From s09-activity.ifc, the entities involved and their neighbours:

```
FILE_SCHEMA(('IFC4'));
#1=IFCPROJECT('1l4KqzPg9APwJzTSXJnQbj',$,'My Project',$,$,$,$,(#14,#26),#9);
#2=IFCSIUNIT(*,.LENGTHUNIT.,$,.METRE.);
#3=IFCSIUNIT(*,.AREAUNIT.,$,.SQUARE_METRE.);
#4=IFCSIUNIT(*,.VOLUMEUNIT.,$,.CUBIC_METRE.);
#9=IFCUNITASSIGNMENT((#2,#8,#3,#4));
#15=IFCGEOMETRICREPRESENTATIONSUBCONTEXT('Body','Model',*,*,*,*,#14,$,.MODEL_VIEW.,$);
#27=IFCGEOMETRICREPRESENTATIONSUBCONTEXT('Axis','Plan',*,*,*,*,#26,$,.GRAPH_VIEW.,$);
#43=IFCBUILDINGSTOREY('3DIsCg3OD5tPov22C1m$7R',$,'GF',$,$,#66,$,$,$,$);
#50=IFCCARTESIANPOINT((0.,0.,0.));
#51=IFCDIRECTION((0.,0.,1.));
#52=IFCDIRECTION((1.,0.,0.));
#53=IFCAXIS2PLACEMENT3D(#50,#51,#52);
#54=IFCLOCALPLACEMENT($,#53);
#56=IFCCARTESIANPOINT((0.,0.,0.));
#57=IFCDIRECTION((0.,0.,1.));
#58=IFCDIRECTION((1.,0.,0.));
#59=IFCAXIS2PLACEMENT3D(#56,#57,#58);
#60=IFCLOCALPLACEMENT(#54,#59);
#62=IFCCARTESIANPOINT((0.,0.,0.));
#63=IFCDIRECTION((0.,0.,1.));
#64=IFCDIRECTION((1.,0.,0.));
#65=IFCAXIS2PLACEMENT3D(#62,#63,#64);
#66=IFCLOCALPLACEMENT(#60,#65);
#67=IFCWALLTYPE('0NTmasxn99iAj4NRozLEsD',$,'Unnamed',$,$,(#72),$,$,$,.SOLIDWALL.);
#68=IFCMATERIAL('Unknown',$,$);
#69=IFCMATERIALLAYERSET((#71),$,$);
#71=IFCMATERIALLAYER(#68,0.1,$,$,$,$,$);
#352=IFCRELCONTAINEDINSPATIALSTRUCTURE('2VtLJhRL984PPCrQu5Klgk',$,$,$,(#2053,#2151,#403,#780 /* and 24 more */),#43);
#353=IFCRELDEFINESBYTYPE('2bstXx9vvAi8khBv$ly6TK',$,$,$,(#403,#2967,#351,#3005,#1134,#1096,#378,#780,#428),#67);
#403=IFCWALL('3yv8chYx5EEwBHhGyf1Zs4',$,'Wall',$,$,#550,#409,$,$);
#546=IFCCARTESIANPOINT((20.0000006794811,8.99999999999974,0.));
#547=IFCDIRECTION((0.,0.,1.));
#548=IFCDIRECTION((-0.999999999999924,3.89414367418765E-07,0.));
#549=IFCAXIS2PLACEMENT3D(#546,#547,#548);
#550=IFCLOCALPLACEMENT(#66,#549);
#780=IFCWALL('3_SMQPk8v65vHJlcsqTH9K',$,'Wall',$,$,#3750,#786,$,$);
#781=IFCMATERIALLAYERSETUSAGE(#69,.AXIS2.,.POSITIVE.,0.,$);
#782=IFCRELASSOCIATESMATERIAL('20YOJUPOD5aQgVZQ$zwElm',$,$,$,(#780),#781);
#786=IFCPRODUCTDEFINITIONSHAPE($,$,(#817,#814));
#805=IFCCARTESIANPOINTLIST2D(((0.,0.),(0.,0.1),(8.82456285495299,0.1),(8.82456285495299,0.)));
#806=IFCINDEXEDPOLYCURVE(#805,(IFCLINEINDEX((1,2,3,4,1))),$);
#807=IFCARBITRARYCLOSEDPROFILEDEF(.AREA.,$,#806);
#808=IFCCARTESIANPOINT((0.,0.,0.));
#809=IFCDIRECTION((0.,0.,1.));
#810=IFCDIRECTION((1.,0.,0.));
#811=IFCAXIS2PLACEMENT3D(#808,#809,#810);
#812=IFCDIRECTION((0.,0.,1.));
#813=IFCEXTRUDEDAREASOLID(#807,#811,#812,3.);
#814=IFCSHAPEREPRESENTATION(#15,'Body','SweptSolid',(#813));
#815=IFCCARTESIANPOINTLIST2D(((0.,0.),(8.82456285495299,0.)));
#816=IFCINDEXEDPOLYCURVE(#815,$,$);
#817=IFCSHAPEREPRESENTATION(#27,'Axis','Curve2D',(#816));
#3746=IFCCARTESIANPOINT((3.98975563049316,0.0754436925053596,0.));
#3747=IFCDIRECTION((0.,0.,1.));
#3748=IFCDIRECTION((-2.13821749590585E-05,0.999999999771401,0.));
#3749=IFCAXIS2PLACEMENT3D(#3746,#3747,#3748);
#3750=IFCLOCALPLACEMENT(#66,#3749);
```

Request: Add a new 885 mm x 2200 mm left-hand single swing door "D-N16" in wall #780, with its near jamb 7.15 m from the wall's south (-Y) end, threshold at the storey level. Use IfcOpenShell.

```python
import numpy as np
import ifcopenshell
import ifcopenshell.api.feature
import ifcopenshell.api.geometry
import ifcopenshell.api.root
import ifcopenshell.api.spatial
import ifcopenshell.geom
import ifcopenshell.util.element
import ifcopenshell.util.placement
import ifcopenshell.util.representation
import ifcopenshell.util.shape
import ifcopenshell.util.unit

model = ifcopenshell.open("s09-activity.ifc")
unit_scale = ifcopenshell.util.unit.calculate_unit_scale(model)
settings = ifcopenshell.geom.settings()


def volume(element):
    """Net volume in cubic metres, openings subtracted."""
    shape = ifcopenshell.geom.create_shape(settings, element)
    return ifcopenshell.util.shape.get_volume(shape.geometry)


wall = model.by_guid("3_SMQPk8v65vHJlcsqTH9K")
storey = ifcopenshell.util.element.get_container(wall, ifc_class="IfcBuildingStorey")
context = ifcopenshell.util.representation.get_context(model, "Model", "Body", "MODEL_VIEW")
before = volume(wall)

width, height, from_end, sill = 0.885, 2.2, 7.15, 0.0  # metres

# The wall runs along its own X axis, and the end named is its -X end.
wall_shape = ifcopenshell.geom.create_shape(settings, wall)
x, y, z = ifcopenshell.util.shape.get_vertices(wall_shape.geometry).T
start = x.min() + from_end
face, thickness = float(y.min()), float(y.max() - y.min())
wall_matrix = ifcopenshell.util.placement.get_local_placement(wall.ObjectPlacement)
level = ifcopenshell.util.placement.get_local_placement(storey.ObjectPlacement)[2, 3]


def in_wall(x, y):
    """Placement at x, y metres in the wall's axes, at sill height."""
    matrix = wall_matrix.copy()
    matrix[:, 3] = wall_matrix @ np.array([x / unit_scale, y / unit_scale, 0.0, 1.0])
    matrix[2, 3] = level + sill / unit_scale
    return matrix


# Opening: a box that overshoots both wall faces by 50 mm.
opening = ifcopenshell.api.root.create_entity(model, ifc_class="IfcOpeningElement", predefined_type="OPENING")
box = ifcopenshell.api.geometry.add_wall_representation(
    model, context=context, length=width, height=height, thickness=thickness + 0.1
)
ifcopenshell.api.geometry.assign_representation(model, product=opening, representation=box)
ifcopenshell.api.geometry.edit_object_placement(model, product=opening, matrix=in_wall(start, face - 0.05), is_si=False)
ifcopenshell.api.feature.add_feature(model, feature=opening, element=wall)

door = ifcopenshell.api.root.create_entity(model, ifc_class="IfcDoor", name="D-N16", predefined_type="DOOR")
door.OverallWidth, door.OverallHeight = width / unit_scale, height / unit_scale
door.OperationType = "SINGLE_SWING_LEFT"
body = ifcopenshell.api.geometry.add_door_representation(
    model,
    context=context,
    overall_width=door.OverallWidth,
    overall_height=door.OverallHeight,
    operation_type="SINGLE_SWING_LEFT",
    lining_properties={"LiningDepth": thickness / unit_scale, "ThresholdDepth": thickness / unit_scale},
)
ifcopenshell.api.geometry.assign_representation(model, product=door, representation=body)
ifcopenshell.api.spatial.assign_container(model, products=[door], relating_structure=storey)
ifcopenshell.api.feature.add_filling(model, opening=opening, element=door)

# The lining spans the wall, so the door starts at the wall face.
ifcopenshell.api.geometry.edit_object_placement(model, product=door, matrix=in_wall(start, face), is_si=False)

after = volume(wall)

print(f"wall volume {before:.3f} -> {after:.3f} m3")

model.write("s09-activity_edited.ifc")
```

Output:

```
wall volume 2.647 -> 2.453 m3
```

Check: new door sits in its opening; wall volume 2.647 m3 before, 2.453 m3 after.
